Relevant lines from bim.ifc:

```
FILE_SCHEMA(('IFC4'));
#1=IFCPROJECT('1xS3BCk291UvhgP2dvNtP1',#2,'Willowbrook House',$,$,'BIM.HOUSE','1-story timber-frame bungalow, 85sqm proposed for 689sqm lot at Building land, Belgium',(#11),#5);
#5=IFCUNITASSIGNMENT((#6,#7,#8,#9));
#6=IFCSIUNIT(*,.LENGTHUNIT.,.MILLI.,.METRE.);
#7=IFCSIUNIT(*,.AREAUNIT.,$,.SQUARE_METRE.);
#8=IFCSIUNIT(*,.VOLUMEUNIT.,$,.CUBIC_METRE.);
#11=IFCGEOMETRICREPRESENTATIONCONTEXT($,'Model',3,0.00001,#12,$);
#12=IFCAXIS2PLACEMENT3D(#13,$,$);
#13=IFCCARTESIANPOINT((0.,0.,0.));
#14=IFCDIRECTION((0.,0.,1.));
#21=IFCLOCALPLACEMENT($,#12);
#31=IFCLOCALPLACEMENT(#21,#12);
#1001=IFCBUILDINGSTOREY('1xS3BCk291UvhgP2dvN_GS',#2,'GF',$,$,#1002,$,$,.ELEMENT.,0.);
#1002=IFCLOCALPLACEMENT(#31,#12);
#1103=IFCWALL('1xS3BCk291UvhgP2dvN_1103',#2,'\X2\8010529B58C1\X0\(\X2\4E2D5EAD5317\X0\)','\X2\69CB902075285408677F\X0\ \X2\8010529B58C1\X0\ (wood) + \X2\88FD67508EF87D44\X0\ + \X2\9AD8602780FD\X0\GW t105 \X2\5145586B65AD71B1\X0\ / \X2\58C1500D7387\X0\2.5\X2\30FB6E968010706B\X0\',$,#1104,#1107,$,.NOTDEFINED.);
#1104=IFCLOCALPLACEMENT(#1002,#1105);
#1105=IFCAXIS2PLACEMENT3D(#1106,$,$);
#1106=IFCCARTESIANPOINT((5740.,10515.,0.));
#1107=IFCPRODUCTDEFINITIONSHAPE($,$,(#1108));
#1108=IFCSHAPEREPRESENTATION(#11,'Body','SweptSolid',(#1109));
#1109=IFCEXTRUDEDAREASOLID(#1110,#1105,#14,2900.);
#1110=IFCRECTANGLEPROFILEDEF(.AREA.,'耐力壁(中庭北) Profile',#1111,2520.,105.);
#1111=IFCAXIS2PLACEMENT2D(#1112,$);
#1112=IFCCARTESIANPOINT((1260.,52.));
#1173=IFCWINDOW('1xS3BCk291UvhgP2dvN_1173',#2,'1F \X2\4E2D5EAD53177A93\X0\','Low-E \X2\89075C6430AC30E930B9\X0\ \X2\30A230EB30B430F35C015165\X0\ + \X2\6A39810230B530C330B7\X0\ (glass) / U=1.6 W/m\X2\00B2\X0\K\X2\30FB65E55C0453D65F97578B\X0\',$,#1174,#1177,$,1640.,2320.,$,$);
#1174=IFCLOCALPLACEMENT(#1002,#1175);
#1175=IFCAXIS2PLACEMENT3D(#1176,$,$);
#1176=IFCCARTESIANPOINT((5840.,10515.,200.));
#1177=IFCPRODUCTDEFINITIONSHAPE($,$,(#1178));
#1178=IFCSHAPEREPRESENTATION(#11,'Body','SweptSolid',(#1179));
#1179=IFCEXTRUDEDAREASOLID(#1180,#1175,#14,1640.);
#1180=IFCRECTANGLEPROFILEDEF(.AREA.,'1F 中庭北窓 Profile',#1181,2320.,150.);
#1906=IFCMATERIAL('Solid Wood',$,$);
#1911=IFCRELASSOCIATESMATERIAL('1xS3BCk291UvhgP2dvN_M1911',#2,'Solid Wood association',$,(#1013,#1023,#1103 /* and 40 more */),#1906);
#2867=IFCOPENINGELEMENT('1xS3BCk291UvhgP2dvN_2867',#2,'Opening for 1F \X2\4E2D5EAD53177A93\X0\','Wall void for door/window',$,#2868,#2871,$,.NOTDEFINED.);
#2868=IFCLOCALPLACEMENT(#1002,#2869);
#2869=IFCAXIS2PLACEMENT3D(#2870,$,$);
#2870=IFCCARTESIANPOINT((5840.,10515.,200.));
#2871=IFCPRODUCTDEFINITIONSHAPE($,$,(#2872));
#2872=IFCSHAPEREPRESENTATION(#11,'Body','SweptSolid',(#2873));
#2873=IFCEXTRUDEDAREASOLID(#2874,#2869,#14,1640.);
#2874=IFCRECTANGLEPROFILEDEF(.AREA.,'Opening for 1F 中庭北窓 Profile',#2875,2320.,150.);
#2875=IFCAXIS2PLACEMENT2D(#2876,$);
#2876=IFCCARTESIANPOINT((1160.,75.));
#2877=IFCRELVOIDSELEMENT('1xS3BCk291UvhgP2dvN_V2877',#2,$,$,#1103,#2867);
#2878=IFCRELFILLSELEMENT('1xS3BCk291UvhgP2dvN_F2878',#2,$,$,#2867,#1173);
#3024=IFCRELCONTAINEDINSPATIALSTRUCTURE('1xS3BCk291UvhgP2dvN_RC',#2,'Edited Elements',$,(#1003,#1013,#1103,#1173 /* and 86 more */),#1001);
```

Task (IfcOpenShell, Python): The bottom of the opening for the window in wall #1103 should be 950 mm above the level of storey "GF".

```python
import numpy as np
import ifcopenshell
import ifcopenshell.api.geometry
import ifcopenshell.geom
import ifcopenshell.util.element
import ifcopenshell.util.placement
import ifcopenshell.util.shape
import ifcopenshell.util.unit

model = ifcopenshell.open("bim.ifc")
unit_scale = ifcopenshell.util.unit.calculate_unit_scale(model)

window = model.by_guid("1xS3BCk291UvhgP2dvN_1173")
opening = window.FillsVoids[0].RelatingOpeningElement
storey = ifcopenshell.util.element.get_container(window, ifc_class="IfcBuildingStorey")
level = ifcopenshell.util.placement.get_local_placement(storey.ObjectPlacement)[2, 3]

# The opening's origin need not be at the sill, so measure its lowest point.
shape = ifcopenshell.geom.create_shape(ifcopenshell.geom.settings(), opening)
bottom = ifcopenshell.util.shape.get_shape_bottom_elevation(shape, shape.geometry) / unit_scale
dz = level + 0.95 / unit_scale - bottom

shift = np.array([0.0, 0.0, dz])
# The window is not placed relative to its opening, so move both.
for product in (opening, window):
    matrix = ifcopenshell.util.placement.get_local_placement(product.ObjectPlacement)
    matrix[:3, 3] += shift
    ifcopenshell.api.geometry.edit_object_placement(model, product=product, matrix=matrix, is_si=False)

print(f"moved by {dz * unit_scale:+.3f} m")

model.write("bim_v2.ifc")
```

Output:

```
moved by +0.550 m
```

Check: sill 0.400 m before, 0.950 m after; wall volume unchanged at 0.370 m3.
